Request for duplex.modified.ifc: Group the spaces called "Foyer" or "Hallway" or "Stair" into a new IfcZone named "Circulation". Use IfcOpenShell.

First a look at what the model holds.

```python
import ifcopenshell

model = ifcopenshell.open("duplex.modified.ifc")
print(model.schema)
seen = {}
for space in model.by_type("IfcSpace"):
    seen[space.LongName] = seen.get(space.LongName, 0) + 1
for name, count in sorted(seen.items(), key=str):
    print(count, "x", name)
print("zones:", [z.Name for z in model.by_type("IfcZone")][:20])
```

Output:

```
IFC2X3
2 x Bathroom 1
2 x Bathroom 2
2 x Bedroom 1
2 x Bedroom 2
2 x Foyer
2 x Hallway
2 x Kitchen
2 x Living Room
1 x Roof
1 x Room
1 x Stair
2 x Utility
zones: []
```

```python
import ifcopenshell
import ifcopenshell.api.group
import ifcopenshell.api.root

model = ifcopenshell.open("duplex.modified.ifc")

names = {"Foyer", "Hallway", "Stair"}
spaces = [s for s in model.by_type("IfcSpace") if s.LongName in names]

zone = ifcopenshell.api.root.create_entity(model, ifc_class="IfcZone", name="Circulation")
ifcopenshell.api.group.assign_group(model, products=spaces, group=zone)
print(len(spaces), "spaces in", zone.Name)

model.write("duplex.modified_edited.ifc")
```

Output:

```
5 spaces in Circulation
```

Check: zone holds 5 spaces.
